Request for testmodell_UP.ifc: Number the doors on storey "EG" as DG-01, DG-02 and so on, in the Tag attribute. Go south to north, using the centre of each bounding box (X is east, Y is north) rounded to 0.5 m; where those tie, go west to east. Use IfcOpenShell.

First a look at what the model holds.

```python
import ifcopenshell
import ifcopenshell.util.element
import ifcopenshell.util.placement

model = ifcopenshell.open("testmodell_UP.ifc")
print(model.schema)
storey = next(s for s in model.by_type("IfcBuildingStorey") if s.Name == "EG")
doors = [e for e in ifcopenshell.util.element.get_decomposition(storey) if e.is_a("IfcDoor")]
for e in sorted(doors, key=lambda e: e.id()):
    origin = ifcopenshell.util.placement.get_local_placement(e.ObjectPlacement)[:3, 3]
    print(e.id(), e.Tag, e.Name, origin.round(2) + 0.0, sep=" | ")
```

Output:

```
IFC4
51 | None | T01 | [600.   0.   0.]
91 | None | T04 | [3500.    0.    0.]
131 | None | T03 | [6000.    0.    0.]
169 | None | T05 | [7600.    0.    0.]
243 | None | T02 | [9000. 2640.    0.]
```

```python
import ifcopenshell
import ifcopenshell.geom
import ifcopenshell.util.element
import ifcopenshell.util.shape

model = ifcopenshell.open("testmodell_UP.ifc")
settings = ifcopenshell.geom.settings()
settings.set("use-world-coords", True)


def centre(element):
    shape = ifcopenshell.geom.create_shape(settings, element)
    return ifcopenshell.util.shape.get_bbox_centroid(shape.geometry)


storey = next(s for s in model.by_type("IfcBuildingStorey") if s.Name == "EG")
doors = [e for e in ifcopenshell.util.element.get_decomposition(storey) if e.is_a("IfcDoor")]

# Insertion points can sit at a corner or the storey origin, so sort by the geometry (in metres).
centres = {e: centre(e) for e in doors}
doors.sort(key=lambda e: (round(centres[e][1] / 0.5), centres[e][0]))

for i, e in enumerate(doors, start=1):
    number = f"DG-{i:02d}"
    e.Tag = number
    print(e.id(), number)

model.write("testmodell_UP_updated.ifc")
```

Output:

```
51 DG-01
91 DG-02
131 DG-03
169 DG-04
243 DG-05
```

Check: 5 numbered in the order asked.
